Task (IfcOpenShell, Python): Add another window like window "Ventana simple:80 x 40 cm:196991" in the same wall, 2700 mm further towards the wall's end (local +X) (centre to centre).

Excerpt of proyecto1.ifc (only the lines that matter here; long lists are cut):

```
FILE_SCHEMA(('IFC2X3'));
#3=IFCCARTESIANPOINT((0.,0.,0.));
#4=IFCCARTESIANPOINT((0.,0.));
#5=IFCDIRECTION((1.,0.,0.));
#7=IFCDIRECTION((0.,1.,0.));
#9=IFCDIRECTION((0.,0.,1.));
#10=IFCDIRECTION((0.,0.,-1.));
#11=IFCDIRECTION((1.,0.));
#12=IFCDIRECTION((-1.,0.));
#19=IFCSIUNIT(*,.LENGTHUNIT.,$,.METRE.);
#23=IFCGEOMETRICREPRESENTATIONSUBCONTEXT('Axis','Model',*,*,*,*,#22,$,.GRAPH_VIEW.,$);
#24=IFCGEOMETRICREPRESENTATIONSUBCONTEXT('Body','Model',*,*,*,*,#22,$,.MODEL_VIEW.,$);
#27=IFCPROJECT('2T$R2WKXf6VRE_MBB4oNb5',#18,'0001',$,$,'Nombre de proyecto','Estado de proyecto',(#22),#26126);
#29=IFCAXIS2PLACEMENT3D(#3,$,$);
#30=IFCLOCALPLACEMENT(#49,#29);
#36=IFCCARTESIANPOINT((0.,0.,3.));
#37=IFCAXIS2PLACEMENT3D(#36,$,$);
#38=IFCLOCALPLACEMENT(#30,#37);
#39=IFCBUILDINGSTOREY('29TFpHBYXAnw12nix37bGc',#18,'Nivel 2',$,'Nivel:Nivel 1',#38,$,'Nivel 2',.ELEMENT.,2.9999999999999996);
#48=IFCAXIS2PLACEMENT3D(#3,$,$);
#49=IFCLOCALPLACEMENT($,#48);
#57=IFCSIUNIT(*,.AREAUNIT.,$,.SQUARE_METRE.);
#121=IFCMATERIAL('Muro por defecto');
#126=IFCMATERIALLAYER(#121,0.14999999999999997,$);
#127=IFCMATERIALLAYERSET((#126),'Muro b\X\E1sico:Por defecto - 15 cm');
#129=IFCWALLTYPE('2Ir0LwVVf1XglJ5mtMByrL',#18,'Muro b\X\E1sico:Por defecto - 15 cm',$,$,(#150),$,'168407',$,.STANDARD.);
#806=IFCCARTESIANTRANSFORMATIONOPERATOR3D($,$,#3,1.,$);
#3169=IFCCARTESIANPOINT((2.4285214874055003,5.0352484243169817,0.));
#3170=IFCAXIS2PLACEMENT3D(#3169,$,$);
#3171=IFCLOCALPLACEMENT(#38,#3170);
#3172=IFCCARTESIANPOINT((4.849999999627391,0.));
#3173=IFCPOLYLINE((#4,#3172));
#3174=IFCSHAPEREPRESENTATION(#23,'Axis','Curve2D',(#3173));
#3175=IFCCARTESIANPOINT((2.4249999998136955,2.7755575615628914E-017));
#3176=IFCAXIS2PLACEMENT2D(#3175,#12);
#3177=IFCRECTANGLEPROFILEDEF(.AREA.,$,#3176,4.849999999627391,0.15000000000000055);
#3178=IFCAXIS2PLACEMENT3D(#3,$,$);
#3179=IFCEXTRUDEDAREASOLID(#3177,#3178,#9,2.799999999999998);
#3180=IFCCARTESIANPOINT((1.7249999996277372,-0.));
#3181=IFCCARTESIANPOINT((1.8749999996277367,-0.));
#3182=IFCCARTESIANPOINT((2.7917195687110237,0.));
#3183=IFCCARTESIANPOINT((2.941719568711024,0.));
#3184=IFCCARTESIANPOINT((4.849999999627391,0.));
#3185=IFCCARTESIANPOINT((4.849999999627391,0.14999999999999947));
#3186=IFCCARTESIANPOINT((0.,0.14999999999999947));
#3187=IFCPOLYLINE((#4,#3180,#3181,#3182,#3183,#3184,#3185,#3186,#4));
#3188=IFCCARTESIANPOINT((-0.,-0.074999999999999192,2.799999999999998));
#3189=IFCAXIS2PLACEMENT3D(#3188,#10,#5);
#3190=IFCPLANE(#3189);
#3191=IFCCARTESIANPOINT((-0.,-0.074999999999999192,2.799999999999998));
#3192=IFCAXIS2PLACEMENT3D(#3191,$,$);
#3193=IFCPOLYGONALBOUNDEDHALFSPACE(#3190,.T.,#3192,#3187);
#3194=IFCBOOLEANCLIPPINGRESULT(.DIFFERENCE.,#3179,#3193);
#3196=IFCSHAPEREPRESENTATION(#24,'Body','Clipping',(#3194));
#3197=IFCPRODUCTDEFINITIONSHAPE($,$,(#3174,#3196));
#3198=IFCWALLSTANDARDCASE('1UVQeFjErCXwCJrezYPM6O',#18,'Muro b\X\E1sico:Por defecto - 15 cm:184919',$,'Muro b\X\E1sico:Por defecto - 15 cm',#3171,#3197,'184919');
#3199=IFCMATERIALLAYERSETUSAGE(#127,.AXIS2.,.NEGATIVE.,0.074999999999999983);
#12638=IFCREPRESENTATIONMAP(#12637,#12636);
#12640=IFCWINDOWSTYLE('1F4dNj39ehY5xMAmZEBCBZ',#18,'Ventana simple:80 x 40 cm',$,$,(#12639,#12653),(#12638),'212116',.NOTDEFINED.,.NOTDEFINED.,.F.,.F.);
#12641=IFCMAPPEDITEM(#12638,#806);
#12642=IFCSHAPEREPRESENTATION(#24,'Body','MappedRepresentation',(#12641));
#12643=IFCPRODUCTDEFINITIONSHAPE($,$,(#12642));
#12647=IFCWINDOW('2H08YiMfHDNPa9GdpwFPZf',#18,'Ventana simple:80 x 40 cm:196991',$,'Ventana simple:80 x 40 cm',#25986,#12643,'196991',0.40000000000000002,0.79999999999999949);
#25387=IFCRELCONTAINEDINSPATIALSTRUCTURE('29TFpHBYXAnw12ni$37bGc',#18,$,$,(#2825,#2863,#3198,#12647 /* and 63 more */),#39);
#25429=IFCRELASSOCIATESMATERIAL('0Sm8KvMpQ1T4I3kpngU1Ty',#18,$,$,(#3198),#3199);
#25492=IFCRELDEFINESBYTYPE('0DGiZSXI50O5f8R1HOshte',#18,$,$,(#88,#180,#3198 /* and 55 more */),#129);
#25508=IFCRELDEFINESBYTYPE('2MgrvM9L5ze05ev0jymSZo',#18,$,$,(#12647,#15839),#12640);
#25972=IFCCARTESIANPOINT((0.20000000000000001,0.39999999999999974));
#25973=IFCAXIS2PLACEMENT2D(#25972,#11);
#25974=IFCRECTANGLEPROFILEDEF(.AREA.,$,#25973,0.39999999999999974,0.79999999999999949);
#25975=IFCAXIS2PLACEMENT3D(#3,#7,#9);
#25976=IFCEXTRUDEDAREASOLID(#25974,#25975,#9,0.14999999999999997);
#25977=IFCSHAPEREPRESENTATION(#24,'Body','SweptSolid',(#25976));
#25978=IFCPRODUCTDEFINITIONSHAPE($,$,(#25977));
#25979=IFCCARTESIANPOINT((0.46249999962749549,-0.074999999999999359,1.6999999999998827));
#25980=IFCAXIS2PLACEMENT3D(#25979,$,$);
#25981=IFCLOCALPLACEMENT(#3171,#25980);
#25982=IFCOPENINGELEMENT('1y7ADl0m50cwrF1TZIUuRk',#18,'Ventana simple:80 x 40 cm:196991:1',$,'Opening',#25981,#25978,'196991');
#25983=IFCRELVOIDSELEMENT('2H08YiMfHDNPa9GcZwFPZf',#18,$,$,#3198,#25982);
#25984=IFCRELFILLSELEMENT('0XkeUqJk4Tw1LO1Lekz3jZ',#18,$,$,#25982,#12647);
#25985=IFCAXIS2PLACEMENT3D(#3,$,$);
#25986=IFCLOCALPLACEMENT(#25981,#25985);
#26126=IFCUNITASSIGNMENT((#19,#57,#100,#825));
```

```python
import ifcopenshell
import ifcopenshell.api.feature
import ifcopenshell.api.geometry
import ifcopenshell.api.root
import ifcopenshell.geom
import ifcopenshell.util.element
import ifcopenshell.util.placement
import ifcopenshell.util.shape
import ifcopenshell.util.unit

model = ifcopenshell.open("proyecto1.ifc")
unit_scale = ifcopenshell.util.unit.calculate_unit_scale(model)
settings = ifcopenshell.geom.settings()


def volume(element):
    """Net volume in cubic metres, openings subtracted."""
    shape = ifcopenshell.geom.create_shape(settings, element)
    return ifcopenshell.util.shape.get_volume(shape.geometry)


def reuse_history(source, copy):
    """copy_class also copies each property set's owner history, people and application; keep the originals."""
    for rel in copy.IsDefinedBy:
        if rel.is_a("IfcRelDefinesByProperties") and (history := rel.RelatingPropertyDefinition.OwnerHistory):
            rel.RelatingPropertyDefinition.OwnerHistory = source.OwnerHistory
            ifcopenshell.util.element.remove_deep2(model, history)


window = model.by_guid("2H08YiMfHDNPa9GdpwFPZf")
opening = window.FillsVoids[0].RelatingOpeningElement
wall = opening.VoidsElements[0].RelatingBuildingElement
before = volume(wall)
shift = ifcopenshell.util.placement.get_local_placement(wall.ObjectPlacement)[:3, 0] * 2.7 / unit_scale

# copy_class copies the void relationship, type, container and properties, but no geometry.
new_opening = ifcopenshell.api.root.copy_class(model, product=opening)
new_opening.Representation = ifcopenshell.util.element.copy_deep(
    model, opening.Representation, exclude=["IfcGeometricRepresentationContext", "IfcRepresentationMap"]
)
new_opening.Name = "Ventana simple:80 x 40 cm"
new_opening.Tag = None
new_window = ifcopenshell.api.root.copy_class(model, product=window)
new_window.Representation = ifcopenshell.util.element.copy_deep(
    model, window.Representation, exclude=["IfcGeometricRepresentationContext", "IfcRepresentationMap"]
)
new_window.Name = "Ventana simple:80 x 40 cm"
new_window.Tag = None
reuse_history(window, new_window)
fills = ifcopenshell.api.feature.add_filling(model, opening=new_opening, element=new_window)
fills.OwnerHistory = new_window.OwnerHistory  # required in IFC2X3

for old, new in ((opening, new_opening), (window, new_window)):
    matrix = ifcopenshell.util.placement.get_local_placement(old.ObjectPlacement)
    matrix[:3, 3] += shift
    ifcopenshell.api.geometry.edit_object_placement(model, product=new, matrix=matrix, is_si=False)

after = volume(wall)

print(f"wall volume {before:.3f} -> {after:.3f} m3")

model.write("proyecto1_edited.ifc")
```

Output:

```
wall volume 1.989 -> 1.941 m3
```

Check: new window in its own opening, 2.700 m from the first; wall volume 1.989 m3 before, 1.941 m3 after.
